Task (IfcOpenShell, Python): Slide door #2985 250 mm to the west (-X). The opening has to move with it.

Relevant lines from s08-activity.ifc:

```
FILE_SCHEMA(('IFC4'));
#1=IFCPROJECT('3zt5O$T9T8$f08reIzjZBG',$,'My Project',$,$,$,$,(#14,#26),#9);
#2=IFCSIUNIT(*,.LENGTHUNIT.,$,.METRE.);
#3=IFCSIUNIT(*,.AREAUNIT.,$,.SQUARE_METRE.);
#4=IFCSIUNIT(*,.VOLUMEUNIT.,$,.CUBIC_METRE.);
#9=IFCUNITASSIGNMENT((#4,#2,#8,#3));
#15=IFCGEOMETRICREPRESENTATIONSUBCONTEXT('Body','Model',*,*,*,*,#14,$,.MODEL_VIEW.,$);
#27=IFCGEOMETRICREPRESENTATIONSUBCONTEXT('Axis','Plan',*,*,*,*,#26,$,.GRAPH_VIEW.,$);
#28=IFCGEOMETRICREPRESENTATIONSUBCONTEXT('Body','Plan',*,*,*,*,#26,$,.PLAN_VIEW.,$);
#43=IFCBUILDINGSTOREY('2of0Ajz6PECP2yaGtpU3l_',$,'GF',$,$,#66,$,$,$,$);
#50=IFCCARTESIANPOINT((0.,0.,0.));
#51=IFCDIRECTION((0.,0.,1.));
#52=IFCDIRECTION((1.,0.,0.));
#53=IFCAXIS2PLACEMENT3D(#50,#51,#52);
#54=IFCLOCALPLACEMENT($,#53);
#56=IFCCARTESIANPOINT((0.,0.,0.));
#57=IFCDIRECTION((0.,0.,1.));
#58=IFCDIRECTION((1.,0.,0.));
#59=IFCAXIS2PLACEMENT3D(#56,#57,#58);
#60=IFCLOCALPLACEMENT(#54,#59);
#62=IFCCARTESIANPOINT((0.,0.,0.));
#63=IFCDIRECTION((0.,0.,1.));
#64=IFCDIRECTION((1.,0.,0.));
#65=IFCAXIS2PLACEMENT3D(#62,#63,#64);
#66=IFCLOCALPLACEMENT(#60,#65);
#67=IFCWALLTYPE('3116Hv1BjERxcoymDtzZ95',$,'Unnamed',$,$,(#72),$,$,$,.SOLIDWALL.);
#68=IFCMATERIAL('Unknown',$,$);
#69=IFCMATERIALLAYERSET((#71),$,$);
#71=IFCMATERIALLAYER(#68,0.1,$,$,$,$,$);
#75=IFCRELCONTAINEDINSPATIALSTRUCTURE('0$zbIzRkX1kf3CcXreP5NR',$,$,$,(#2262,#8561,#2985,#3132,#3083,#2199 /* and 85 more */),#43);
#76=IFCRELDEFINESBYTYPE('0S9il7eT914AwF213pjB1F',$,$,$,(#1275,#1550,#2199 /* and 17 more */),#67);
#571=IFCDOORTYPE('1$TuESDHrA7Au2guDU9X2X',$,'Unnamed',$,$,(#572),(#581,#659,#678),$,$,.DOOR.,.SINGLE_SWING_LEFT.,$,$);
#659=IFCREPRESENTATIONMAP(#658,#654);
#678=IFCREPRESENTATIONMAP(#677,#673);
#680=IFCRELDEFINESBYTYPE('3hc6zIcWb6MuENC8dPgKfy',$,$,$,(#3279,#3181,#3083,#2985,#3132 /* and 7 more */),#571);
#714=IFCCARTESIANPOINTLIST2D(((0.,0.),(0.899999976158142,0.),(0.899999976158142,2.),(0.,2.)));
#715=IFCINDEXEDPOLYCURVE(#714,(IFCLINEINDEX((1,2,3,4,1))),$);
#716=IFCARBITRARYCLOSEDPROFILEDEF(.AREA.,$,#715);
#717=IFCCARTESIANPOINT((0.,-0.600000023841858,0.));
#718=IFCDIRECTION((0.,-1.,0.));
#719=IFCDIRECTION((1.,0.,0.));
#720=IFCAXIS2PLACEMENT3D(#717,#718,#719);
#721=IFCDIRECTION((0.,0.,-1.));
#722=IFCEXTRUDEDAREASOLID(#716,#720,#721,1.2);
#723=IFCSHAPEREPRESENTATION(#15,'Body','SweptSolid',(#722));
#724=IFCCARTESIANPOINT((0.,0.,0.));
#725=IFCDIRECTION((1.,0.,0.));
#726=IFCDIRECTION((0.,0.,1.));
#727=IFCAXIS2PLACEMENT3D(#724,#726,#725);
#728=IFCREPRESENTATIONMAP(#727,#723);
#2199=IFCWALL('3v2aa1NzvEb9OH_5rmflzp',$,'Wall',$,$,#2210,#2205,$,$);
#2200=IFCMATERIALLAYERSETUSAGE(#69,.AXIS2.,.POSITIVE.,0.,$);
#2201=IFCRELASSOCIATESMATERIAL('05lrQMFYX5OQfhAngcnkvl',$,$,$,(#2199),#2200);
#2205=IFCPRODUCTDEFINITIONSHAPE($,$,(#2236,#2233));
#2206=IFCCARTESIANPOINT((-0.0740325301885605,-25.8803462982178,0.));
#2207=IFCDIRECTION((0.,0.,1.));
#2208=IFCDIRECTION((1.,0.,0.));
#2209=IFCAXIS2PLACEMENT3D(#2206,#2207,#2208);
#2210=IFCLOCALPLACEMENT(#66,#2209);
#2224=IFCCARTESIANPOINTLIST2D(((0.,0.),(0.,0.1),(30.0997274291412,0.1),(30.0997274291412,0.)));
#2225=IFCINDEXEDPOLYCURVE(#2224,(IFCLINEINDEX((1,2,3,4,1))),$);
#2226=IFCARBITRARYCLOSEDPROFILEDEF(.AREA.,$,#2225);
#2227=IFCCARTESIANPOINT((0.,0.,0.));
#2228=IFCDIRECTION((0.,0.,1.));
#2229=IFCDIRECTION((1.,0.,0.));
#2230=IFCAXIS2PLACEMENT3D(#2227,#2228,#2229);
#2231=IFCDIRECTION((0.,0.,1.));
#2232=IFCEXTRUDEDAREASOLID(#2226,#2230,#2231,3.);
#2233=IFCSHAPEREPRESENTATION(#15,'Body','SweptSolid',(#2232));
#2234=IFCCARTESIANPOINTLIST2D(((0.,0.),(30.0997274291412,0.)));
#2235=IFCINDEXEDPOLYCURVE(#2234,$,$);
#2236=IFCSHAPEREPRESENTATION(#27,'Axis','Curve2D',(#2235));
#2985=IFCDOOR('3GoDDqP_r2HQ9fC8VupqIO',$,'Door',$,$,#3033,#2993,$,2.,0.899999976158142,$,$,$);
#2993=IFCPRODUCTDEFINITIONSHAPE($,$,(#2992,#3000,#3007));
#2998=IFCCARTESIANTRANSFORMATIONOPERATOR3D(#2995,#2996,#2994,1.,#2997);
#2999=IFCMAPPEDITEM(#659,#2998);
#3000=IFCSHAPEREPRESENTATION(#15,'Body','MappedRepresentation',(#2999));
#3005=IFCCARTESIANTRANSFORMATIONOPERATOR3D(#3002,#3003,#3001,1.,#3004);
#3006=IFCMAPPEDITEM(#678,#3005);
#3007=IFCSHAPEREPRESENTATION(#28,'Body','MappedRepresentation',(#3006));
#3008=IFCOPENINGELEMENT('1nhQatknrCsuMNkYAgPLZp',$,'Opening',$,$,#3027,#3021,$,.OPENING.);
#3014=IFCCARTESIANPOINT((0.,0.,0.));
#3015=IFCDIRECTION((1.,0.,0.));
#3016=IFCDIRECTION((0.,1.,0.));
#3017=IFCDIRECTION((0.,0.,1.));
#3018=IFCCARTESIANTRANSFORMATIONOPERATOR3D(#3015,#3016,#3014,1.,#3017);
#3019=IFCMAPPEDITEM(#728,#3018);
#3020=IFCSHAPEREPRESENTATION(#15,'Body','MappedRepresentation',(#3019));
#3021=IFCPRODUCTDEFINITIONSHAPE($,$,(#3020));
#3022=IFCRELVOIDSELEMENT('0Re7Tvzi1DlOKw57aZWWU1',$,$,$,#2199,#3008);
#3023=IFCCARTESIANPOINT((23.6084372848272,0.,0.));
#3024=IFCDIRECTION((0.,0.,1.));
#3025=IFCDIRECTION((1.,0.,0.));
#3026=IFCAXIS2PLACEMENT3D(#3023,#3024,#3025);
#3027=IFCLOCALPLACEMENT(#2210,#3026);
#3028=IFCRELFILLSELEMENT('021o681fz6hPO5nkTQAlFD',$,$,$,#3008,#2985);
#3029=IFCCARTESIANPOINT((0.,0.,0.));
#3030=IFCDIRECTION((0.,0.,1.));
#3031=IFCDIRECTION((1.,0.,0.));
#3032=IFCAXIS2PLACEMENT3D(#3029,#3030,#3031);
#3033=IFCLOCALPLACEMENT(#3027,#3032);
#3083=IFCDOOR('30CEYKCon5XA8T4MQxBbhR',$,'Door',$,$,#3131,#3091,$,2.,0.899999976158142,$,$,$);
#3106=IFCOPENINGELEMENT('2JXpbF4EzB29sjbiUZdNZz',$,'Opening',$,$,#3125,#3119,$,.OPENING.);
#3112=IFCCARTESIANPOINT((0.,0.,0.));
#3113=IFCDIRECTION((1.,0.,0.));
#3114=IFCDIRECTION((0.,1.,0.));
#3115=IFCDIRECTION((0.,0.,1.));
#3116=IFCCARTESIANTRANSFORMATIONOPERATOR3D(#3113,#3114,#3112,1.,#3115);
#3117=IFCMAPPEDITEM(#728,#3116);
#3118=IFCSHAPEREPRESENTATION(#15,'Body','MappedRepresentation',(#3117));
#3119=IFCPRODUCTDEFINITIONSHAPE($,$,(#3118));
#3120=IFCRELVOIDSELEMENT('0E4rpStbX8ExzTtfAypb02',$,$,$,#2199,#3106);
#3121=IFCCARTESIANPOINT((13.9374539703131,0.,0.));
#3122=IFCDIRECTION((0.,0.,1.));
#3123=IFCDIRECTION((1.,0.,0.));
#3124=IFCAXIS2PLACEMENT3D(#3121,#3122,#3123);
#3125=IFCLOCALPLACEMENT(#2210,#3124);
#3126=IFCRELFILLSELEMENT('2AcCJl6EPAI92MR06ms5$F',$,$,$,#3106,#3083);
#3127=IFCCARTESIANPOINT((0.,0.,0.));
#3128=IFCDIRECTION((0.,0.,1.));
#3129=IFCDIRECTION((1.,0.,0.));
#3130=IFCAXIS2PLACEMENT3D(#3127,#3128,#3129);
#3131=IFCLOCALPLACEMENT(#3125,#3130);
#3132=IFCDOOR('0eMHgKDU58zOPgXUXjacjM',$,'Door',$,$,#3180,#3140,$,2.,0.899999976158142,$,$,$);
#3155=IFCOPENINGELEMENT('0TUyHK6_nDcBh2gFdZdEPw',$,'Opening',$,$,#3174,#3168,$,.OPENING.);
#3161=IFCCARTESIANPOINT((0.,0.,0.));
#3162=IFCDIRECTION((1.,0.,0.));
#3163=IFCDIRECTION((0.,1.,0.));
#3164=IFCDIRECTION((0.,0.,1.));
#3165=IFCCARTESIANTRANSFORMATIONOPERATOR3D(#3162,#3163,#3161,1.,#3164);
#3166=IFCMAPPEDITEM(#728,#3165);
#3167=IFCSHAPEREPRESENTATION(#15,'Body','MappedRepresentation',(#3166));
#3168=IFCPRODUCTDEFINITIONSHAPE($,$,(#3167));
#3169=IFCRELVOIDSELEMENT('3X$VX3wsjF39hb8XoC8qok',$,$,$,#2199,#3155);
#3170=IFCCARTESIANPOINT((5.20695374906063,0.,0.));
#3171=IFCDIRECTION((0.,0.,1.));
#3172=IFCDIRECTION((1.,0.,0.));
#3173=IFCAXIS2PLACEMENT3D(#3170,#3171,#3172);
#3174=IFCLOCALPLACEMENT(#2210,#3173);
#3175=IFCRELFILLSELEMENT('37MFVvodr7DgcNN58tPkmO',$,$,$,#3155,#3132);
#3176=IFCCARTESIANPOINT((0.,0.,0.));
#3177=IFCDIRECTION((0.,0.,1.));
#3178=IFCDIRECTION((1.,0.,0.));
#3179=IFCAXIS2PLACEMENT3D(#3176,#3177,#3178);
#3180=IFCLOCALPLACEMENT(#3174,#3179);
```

```python
import ifcopenshell
import ifcopenshell.api.geometry
import ifcopenshell.util.placement

model = ifcopenshell.open("s08-activity.ifc")

door = model.by_guid("3GoDDqP_r2HQ9fC8VupqIO")
opening = door.FillsVoids[0].RelatingOpeningElement
wall = opening.VoidsElements[0].RelatingBuildingElement

wall_matrix = ifcopenshell.util.placement.get_local_placement(wall.ObjectPlacement)
shift = wall_matrix[:3, 0] * -0.25
before = ifcopenshell.util.placement.get_local_placement(door.ObjectPlacement)[:3, 3].copy()

# The door is placed relative to its opening, so it follows when the opening moves.
matrix = ifcopenshell.util.placement.get_local_placement(opening.ObjectPlacement)
matrix[:3, 3] += shift
ifcopenshell.api.geometry.edit_object_placement(
    model, product=opening, matrix=matrix, is_si=False, should_transform_children=True
)

after = ifcopenshell.util.placement.get_local_placement(door.ObjectPlacement)[:3, 3]
print("door moved by", (after - before).round(3) + 0.0)

model.write("s08-activity_v2.ifc")
```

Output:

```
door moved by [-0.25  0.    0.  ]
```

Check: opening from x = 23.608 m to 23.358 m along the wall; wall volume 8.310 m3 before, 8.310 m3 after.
